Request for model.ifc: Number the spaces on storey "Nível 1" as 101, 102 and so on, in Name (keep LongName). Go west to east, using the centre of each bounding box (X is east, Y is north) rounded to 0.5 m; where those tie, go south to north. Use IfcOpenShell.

First a look at what the model holds.

```python
import ifcopenshell
import ifcopenshell.util.element
import ifcopenshell.util.placement

model = ifcopenshell.open("model.ifc")
print(model.schema)
storey = next(s for s in model.by_type("IfcBuildingStorey") if s.Name == "Nível 1")
spaces = [e for e in ifcopenshell.util.element.get_decomposition(storey) if e.is_a("IfcSpace")]
for e in sorted(spaces, key=lambda e: e.id()):
    origin = ifcopenshell.util.placement.get_local_placement(e.ObjectPlacement)[:3, 3]
    print(e.id(), e.Name, e.LongName, origin.round(2) + 0.0, sep=" | ")
```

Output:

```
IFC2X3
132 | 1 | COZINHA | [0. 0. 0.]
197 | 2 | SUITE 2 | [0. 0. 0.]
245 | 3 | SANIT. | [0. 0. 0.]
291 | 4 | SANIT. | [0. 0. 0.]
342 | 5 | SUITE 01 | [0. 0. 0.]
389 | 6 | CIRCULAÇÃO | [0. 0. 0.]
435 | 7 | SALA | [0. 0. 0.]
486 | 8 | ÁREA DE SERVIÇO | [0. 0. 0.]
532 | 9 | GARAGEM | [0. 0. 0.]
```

```python
import ifcopenshell
import ifcopenshell.geom
import ifcopenshell.util.element
import ifcopenshell.util.shape

model = ifcopenshell.open("model.ifc")
settings = ifcopenshell.geom.settings()
settings.set("use-world-coords", True)


def centre(element):
    shape = ifcopenshell.geom.create_shape(settings, element)
    return ifcopenshell.util.shape.get_bbox_centroid(shape.geometry)


storey = next(s for s in model.by_type("IfcBuildingStorey") if s.Name == "Nível 1")
spaces = [e for e in ifcopenshell.util.element.get_decomposition(storey) if e.is_a("IfcSpace")]

# Insertion points can sit at a corner or the storey origin, so sort by the geometry (in metres).
centres = {e: centre(e) for e in spaces}
spaces.sort(key=lambda e: (round(centres[e][0] / 0.5), centres[e][1]))

for i, e in enumerate(spaces, start=1):
    number = f"1{i:02d}"
    e.Name = number
    print(e.id(), number)

model.write("model-out.ifc")
```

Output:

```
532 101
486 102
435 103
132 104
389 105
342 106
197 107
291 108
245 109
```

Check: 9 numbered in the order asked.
